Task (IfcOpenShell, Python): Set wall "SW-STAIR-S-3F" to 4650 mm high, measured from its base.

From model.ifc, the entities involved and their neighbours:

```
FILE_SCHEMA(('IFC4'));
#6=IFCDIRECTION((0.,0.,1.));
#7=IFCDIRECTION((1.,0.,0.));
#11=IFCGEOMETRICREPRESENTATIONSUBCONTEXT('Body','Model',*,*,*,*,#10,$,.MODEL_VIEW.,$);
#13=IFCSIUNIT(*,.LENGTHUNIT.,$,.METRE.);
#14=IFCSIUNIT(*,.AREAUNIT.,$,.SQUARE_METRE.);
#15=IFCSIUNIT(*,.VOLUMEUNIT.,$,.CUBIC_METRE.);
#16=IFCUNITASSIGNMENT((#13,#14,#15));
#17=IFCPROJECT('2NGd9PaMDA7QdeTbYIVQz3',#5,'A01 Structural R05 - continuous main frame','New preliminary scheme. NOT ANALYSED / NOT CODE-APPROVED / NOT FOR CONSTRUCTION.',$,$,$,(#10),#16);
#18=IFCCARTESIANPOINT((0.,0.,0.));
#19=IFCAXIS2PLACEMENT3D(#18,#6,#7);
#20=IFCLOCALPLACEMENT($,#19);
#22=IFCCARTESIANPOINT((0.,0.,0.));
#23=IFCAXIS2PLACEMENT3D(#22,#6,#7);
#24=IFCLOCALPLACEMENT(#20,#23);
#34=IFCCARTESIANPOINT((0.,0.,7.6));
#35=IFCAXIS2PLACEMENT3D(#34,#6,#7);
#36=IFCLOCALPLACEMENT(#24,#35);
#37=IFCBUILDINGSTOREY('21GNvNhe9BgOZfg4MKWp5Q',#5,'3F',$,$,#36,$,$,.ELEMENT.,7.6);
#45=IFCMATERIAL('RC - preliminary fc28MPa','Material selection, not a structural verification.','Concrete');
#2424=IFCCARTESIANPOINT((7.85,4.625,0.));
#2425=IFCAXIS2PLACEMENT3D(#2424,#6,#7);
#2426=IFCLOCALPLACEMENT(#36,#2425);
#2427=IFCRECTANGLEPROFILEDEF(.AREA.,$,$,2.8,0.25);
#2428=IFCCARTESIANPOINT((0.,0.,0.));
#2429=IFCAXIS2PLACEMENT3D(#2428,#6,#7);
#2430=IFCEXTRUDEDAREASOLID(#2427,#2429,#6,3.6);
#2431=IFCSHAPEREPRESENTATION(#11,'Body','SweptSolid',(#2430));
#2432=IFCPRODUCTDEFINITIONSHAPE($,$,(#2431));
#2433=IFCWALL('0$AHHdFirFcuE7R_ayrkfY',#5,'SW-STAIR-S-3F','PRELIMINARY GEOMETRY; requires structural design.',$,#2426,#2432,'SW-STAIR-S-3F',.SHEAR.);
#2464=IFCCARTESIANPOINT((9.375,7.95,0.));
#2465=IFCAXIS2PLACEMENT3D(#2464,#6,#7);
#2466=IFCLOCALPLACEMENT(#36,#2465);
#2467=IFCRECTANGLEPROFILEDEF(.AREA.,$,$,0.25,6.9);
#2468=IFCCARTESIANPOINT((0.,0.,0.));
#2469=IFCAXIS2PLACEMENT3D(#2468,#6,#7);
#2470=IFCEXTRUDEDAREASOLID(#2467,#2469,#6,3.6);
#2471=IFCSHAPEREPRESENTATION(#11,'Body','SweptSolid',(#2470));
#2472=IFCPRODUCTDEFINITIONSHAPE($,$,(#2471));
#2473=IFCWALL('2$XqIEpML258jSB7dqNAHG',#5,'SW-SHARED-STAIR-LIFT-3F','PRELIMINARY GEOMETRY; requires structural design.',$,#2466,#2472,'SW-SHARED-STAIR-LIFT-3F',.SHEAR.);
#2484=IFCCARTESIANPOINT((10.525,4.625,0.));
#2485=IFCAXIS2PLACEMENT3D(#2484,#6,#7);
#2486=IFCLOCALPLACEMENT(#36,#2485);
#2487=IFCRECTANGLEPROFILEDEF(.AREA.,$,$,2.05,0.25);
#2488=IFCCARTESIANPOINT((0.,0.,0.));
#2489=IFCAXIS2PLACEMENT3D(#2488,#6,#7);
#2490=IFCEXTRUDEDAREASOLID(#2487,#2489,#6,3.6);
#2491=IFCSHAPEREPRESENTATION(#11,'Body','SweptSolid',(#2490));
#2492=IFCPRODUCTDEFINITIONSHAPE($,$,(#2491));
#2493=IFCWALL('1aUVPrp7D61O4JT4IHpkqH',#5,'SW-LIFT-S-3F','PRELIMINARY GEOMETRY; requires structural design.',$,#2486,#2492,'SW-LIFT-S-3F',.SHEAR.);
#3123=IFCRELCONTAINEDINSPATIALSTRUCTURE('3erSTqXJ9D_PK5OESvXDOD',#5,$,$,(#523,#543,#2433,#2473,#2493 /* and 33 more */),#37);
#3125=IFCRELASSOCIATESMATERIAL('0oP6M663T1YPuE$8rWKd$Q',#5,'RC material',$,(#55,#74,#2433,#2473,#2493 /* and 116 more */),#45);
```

```python
import ifcopenshell
import ifcopenshell.geom
import ifcopenshell.util.representation
import ifcopenshell.util.shape

model = ifcopenshell.open("model.ifc")
settings = ifcopenshell.geom.settings()


def volume(element):
    """Net volume in cubic metres, openings subtracted."""
    shape = ifcopenshell.geom.create_shape(settings, element)
    return ifcopenshell.util.shape.get_volume(shape.geometry)


wall = model.by_id(2433)
before = volume(wall)

body = ifcopenshell.util.representation.get_representation(wall, "Model", "Body")
solid = body.Items[0]
old_height = solid.Depth
solid.Depth = 4.65
after = volume(wall)

print(f"height {old_height:g} -> {solid.Depth:g}, volume {before:.3f} -> {after:.3f} m3")

model.write("model_rev.ifc")
```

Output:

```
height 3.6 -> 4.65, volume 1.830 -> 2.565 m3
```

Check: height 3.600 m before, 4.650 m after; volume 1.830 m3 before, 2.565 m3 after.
